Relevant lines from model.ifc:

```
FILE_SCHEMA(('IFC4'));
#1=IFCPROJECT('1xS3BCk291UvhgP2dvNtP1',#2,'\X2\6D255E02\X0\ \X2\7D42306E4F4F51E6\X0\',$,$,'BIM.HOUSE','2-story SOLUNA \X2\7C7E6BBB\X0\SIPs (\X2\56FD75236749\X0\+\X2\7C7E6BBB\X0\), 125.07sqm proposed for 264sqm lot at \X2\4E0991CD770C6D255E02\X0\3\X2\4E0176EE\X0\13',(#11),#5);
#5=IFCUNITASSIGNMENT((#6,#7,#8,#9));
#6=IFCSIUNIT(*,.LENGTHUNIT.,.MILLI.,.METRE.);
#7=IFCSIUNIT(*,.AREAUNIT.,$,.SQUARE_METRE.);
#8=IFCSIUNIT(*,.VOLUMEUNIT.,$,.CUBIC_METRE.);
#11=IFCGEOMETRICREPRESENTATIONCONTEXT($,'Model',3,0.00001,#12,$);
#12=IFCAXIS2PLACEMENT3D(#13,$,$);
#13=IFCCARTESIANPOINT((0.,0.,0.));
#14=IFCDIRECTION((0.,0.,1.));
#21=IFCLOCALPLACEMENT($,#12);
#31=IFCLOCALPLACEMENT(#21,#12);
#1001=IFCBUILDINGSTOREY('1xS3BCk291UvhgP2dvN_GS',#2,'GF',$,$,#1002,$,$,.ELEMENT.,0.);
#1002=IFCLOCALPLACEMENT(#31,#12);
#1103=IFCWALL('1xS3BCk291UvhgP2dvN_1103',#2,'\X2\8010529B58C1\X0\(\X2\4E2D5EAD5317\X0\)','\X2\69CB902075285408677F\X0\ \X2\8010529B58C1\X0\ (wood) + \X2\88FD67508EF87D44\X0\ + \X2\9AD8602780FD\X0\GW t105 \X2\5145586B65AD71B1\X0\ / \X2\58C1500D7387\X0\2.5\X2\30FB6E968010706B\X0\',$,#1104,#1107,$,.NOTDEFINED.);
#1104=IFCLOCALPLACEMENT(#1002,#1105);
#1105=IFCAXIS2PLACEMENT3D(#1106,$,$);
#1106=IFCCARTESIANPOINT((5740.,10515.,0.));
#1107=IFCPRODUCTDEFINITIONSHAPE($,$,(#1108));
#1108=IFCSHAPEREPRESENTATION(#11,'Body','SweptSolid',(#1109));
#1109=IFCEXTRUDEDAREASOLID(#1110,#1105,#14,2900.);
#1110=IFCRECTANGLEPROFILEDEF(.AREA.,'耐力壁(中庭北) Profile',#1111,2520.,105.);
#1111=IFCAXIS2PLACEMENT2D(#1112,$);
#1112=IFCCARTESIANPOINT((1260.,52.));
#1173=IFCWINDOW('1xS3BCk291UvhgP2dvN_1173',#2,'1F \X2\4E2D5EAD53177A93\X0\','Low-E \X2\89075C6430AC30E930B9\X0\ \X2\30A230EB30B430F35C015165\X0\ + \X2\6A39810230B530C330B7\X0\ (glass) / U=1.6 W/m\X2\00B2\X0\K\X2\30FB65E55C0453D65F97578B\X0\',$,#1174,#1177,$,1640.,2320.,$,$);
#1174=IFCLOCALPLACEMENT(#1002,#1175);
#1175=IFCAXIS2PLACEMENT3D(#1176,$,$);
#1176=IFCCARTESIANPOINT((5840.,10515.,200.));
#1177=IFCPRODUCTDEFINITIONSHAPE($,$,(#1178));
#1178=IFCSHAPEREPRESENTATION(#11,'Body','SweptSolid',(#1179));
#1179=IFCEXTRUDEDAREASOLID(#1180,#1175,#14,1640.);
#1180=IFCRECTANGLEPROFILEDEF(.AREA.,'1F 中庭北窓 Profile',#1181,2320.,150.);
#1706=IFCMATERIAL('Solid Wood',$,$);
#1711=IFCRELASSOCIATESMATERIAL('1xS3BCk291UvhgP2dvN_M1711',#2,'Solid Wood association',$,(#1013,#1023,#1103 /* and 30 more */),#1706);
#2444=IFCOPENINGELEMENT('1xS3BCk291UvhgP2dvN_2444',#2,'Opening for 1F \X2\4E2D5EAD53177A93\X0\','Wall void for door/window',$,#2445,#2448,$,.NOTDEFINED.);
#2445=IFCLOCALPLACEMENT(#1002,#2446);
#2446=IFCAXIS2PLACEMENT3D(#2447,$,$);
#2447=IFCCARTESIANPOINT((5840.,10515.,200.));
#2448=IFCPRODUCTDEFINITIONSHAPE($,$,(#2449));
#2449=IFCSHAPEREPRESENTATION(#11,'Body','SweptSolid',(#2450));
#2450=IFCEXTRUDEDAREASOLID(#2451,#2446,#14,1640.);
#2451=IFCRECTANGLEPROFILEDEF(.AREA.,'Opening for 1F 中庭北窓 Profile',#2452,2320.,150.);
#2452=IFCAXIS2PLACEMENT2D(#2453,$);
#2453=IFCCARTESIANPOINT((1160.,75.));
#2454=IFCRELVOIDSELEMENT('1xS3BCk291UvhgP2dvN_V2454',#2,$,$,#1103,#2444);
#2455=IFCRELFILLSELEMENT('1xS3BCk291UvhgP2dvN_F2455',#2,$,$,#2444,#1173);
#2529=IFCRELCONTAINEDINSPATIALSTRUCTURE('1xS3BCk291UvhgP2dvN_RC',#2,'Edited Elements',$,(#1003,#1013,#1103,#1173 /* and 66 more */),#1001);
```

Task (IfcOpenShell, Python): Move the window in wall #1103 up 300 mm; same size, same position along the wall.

```python
import numpy as np
import ifcopenshell
import ifcopenshell.api.geometry
import ifcopenshell.util.placement
import ifcopenshell.util.unit

model = ifcopenshell.open("model.ifc")
unit_scale = ifcopenshell.util.unit.calculate_unit_scale(model)

window = model.by_guid("1xS3BCk291UvhgP2dvN_1173")
opening = window.FillsVoids[0].RelatingOpeningElement
dz = 0.3 / unit_scale

shift = np.array([0.0, 0.0, dz])
# The window is not placed relative to its opening, so move both.
for product in (opening, window):
    matrix = ifcopenshell.util.placement.get_local_placement(product.ObjectPlacement)
    matrix[:3, 3] += shift
    ifcopenshell.api.geometry.edit_object_placement(model, product=product, matrix=matrix, is_si=False)

print(f"moved by {dz * unit_scale:+.3f} m")

model.write("model_updated.ifc")
```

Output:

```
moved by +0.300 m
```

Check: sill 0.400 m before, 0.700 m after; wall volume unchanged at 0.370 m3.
